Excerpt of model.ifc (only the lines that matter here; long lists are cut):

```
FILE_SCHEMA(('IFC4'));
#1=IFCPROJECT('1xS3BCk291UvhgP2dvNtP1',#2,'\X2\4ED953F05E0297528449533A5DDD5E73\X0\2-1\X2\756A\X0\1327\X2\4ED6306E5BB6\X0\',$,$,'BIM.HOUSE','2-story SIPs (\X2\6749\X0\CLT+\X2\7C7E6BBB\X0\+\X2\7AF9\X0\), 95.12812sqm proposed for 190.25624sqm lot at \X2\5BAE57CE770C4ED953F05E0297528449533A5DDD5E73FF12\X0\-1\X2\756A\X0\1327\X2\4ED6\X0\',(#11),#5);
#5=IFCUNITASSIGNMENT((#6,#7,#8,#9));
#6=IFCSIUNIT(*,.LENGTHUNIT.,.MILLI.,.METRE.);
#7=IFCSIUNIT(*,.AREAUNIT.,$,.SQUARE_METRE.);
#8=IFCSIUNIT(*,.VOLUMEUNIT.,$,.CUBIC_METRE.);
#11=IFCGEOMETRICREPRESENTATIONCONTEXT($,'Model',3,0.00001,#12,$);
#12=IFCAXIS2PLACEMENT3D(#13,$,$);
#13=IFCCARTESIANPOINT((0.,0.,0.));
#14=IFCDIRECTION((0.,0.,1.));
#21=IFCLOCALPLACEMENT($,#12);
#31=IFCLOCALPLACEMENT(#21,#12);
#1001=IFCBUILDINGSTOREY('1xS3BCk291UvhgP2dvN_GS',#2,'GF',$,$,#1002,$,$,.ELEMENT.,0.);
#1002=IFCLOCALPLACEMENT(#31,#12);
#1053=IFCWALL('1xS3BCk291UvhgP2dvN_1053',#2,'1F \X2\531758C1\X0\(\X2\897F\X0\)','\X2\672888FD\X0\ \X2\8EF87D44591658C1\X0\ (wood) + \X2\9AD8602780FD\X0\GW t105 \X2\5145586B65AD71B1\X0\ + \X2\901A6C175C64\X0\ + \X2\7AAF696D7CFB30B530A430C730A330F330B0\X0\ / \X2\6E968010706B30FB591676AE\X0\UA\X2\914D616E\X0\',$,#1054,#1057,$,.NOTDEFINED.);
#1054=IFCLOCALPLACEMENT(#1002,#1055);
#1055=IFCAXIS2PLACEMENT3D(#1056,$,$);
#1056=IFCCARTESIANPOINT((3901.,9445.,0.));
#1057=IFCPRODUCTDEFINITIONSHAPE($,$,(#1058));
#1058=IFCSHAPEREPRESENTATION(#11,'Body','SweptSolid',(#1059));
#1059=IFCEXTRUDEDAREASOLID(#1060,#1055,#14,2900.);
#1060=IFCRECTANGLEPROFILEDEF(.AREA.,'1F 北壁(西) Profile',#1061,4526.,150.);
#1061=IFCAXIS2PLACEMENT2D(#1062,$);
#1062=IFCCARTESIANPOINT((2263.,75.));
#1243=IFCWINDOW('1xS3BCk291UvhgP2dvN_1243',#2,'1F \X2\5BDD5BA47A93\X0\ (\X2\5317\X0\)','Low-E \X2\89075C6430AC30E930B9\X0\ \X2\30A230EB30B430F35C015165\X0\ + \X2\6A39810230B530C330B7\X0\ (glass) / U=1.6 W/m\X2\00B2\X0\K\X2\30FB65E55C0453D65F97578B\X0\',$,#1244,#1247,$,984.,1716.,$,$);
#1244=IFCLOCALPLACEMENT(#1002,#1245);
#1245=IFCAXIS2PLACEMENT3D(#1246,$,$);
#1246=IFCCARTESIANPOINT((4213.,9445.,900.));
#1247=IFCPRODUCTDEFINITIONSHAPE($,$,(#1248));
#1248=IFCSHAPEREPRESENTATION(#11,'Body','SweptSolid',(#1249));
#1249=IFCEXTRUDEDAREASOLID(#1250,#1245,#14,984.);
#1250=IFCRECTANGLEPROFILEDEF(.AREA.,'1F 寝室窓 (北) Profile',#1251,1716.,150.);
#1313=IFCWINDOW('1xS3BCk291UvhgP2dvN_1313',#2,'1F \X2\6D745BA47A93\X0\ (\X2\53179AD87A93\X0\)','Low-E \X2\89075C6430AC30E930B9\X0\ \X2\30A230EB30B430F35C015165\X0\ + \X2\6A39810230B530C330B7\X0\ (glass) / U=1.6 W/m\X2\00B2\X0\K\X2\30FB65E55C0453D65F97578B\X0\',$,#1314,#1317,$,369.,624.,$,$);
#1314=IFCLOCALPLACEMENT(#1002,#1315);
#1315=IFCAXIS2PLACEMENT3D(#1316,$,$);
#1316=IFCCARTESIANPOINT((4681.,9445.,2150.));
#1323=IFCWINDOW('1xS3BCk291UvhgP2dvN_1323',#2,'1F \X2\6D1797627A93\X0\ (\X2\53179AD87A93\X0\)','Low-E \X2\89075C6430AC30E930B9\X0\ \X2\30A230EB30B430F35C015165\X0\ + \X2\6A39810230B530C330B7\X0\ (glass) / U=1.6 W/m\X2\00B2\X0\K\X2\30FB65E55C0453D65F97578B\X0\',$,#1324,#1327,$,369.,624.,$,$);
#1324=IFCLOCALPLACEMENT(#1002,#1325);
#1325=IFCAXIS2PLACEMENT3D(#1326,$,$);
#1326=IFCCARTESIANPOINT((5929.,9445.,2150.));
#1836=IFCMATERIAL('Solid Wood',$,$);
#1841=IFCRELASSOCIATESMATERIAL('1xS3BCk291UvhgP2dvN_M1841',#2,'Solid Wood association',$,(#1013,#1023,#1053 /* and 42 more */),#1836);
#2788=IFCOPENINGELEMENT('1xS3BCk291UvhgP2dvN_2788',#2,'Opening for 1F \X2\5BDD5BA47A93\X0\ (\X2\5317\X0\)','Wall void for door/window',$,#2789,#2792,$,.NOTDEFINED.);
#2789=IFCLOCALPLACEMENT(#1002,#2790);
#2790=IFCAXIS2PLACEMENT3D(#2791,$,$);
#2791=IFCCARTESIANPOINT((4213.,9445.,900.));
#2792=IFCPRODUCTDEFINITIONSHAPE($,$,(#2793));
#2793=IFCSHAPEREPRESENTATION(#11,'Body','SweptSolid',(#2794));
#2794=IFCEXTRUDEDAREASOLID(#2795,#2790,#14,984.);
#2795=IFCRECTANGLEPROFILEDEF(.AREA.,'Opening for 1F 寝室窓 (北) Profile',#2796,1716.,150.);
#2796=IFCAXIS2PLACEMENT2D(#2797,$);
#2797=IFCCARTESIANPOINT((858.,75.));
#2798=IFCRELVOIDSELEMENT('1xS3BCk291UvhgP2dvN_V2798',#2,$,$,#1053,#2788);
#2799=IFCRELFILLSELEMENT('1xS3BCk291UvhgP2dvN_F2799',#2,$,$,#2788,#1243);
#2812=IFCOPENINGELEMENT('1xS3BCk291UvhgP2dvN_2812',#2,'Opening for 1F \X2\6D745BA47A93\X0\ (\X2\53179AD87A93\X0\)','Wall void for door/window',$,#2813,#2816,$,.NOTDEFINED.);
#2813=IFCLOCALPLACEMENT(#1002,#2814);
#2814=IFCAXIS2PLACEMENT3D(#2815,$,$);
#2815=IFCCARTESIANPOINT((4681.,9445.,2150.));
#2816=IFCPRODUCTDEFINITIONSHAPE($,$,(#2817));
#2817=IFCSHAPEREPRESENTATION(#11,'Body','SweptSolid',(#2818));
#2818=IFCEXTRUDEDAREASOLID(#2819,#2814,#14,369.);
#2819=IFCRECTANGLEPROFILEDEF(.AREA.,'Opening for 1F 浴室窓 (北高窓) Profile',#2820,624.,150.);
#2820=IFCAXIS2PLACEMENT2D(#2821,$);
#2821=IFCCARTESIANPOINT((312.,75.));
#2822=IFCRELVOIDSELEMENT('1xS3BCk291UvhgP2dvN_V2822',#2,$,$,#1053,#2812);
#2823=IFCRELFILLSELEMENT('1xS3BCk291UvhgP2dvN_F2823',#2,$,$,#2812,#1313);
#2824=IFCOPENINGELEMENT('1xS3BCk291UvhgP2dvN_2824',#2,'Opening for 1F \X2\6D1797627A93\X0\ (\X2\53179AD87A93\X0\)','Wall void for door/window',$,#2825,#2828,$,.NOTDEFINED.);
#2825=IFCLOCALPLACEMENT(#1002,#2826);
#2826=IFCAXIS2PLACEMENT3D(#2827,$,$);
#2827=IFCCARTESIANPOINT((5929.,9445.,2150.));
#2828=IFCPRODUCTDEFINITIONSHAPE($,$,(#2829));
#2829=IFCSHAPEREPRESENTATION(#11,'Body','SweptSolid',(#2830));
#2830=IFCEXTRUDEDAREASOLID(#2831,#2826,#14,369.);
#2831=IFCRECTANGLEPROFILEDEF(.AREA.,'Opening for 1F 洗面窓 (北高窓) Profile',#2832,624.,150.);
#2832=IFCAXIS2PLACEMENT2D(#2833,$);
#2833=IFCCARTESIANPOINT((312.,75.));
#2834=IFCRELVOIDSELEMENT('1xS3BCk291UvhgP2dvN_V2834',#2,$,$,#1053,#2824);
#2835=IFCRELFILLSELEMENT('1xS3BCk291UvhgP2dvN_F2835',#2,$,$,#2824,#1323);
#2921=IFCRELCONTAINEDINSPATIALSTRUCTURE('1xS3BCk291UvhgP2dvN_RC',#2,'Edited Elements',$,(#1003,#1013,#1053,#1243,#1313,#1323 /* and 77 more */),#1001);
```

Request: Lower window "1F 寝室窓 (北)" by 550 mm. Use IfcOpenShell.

```python
import numpy as np
import ifcopenshell
import ifcopenshell.api.geometry
import ifcopenshell.util.placement
import ifcopenshell.util.unit

model = ifcopenshell.open("model.ifc")
unit_scale = ifcopenshell.util.unit.calculate_unit_scale(model)

window = model.by_id(1243)
opening = window.FillsVoids[0].RelatingOpeningElement
dz = -0.55 / unit_scale

shift = np.array([0.0, 0.0, dz])
# The window is not placed relative to its opening, so move both.
for product in (opening, window):
    matrix = ifcopenshell.util.placement.get_local_placement(product.ObjectPlacement)
    matrix[:3, 3] += shift
    ifcopenshell.api.geometry.edit_object_placement(model, product=product, matrix=matrix, is_si=False)

print(f"moved by {dz * unit_scale:+.3f} m")

model.write("model_rev.ifc")
```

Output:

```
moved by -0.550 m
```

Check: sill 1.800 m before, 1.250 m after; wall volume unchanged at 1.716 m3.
